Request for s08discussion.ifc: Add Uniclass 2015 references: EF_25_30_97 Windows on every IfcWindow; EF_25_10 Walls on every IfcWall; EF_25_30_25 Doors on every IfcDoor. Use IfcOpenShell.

First a look at what the model holds.

```python
import ifcopenshell

model = ifcopenshell.open("s08discussion.ifc")
print(model.schema)
print("classifications:", [c.Name for c in model.by_type("IfcClassification")])
for ifc_class in ("IfcDoor", "IfcRoof", "IfcStair", "IfcWall", "IfcWindow"):
    print(ifc_class, len(model.by_type(ifc_class)))
```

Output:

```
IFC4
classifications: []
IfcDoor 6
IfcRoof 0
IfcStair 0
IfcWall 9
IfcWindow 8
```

```python
import ifcopenshell
import ifcopenshell.api.classification

model = ifcopenshell.open("s08discussion.ifc")

system = ifcopenshell.api.classification.add_classification(model, classification="Uniclass 2015")

codes = {
    "IfcWindow": ("EF_25_30_97", "Windows"),
    "IfcWall": ("EF_25_10", "Walls"),
    "IfcDoor": ("EF_25_30_25", "Doors"),
}
for ifc_class, (code, name) in codes.items():
    products = model.by_type(ifc_class)
    ifcopenshell.api.classification.add_reference(
        model, products=products, classification=system, identification=code, name=name
    )
    print(code, len(products))

model.write("s08discussion-out.ifc")
```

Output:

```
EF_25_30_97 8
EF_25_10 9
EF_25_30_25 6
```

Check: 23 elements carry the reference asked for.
